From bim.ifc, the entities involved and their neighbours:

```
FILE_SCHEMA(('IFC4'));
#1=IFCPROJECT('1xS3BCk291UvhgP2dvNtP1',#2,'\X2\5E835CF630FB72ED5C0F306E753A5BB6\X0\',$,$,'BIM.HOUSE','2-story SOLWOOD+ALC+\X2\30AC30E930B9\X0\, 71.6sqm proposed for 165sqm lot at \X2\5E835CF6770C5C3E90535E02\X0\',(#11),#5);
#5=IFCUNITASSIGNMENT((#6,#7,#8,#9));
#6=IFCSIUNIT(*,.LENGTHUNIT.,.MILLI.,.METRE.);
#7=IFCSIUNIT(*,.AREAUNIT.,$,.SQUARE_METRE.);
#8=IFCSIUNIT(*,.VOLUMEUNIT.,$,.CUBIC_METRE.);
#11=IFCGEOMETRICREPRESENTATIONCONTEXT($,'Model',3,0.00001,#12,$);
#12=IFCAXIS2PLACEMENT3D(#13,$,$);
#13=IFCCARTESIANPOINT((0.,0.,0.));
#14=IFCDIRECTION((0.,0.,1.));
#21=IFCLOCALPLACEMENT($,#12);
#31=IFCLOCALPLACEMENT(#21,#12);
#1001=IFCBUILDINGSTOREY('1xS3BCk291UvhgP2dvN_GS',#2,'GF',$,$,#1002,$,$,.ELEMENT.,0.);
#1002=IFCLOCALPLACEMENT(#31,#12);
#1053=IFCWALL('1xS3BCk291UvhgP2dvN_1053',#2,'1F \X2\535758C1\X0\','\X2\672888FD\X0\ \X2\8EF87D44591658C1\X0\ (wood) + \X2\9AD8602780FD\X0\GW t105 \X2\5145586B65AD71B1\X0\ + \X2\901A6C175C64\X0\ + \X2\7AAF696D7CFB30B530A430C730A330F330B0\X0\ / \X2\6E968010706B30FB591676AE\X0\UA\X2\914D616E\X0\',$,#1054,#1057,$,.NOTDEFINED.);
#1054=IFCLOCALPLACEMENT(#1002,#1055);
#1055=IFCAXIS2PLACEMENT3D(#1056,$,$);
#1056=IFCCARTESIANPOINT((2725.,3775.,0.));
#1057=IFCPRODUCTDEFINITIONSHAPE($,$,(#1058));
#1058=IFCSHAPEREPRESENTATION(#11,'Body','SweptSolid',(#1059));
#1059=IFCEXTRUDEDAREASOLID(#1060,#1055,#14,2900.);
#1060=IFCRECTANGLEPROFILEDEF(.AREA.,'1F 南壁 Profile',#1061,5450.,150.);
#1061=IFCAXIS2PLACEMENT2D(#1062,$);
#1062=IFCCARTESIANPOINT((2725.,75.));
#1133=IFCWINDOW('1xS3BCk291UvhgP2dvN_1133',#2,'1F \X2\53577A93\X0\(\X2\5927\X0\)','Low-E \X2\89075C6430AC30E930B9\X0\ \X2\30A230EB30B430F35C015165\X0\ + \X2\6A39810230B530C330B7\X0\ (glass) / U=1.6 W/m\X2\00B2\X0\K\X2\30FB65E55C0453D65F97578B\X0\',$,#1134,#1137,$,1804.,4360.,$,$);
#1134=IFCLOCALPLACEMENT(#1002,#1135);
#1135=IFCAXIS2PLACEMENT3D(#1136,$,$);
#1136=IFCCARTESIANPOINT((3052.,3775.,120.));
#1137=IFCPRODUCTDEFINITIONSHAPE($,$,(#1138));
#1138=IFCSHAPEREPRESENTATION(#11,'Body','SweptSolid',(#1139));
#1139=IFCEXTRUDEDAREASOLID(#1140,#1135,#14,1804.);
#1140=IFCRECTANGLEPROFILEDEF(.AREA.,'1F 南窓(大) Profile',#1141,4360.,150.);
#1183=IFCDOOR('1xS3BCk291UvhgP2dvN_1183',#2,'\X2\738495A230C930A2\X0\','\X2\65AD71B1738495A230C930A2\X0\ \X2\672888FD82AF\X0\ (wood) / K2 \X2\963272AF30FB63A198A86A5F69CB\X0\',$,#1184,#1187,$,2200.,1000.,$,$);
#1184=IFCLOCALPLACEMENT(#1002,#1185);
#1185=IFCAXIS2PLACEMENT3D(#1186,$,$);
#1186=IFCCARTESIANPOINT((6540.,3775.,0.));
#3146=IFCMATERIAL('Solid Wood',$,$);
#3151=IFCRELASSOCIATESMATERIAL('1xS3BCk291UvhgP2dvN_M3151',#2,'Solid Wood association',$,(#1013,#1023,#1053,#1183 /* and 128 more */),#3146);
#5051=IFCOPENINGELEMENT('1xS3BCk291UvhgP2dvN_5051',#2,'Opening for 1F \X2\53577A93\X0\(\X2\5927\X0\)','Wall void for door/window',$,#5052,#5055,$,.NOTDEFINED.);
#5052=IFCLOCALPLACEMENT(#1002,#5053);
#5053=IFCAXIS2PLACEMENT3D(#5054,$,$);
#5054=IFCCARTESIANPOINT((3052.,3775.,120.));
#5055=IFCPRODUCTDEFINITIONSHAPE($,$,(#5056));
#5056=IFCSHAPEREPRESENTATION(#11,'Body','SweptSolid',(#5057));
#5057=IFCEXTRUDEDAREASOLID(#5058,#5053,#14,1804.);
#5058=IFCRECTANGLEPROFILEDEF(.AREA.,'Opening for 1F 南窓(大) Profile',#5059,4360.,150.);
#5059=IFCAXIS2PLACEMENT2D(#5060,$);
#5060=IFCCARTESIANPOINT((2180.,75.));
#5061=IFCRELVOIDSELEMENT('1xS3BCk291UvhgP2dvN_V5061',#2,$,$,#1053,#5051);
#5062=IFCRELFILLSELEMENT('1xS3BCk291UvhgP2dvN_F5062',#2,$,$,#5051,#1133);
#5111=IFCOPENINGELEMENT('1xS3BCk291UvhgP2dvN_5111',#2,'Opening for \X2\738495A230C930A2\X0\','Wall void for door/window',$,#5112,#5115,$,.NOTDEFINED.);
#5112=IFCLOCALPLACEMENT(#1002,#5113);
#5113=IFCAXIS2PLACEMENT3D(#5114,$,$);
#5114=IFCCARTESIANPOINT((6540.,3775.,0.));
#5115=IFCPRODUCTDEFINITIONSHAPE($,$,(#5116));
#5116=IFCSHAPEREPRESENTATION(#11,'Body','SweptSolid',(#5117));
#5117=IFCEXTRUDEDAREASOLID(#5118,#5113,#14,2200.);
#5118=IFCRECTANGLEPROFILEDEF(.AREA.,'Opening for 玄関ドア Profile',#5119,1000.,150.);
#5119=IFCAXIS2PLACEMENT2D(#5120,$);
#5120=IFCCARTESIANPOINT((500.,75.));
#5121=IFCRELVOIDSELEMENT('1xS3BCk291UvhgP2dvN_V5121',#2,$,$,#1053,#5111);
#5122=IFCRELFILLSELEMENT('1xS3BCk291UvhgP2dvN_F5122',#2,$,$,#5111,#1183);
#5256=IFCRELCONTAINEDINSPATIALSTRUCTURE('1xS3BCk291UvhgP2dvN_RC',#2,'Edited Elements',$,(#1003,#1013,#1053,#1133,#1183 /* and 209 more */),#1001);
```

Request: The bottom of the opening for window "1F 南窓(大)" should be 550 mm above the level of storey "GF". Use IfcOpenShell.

```python
import numpy as np
import ifcopenshell
import ifcopenshell.api.geometry
import ifcopenshell.geom
import ifcopenshell.util.element
import ifcopenshell.util.placement
import ifcopenshell.util.shape
import ifcopenshell.util.unit

model = ifcopenshell.open("bim.ifc")
unit_scale = ifcopenshell.util.unit.calculate_unit_scale(model)

window = model.by_guid("1xS3BCk291UvhgP2dvN_1133")
opening = window.FillsVoids[0].RelatingOpeningElement
storey = ifcopenshell.util.element.get_container(window, ifc_class="IfcBuildingStorey")
level = ifcopenshell.util.placement.get_local_placement(storey.ObjectPlacement)[2, 3]

# The opening's origin need not be at the sill, so measure its lowest point.
shape = ifcopenshell.geom.create_shape(ifcopenshell.geom.settings(), opening)
bottom = ifcopenshell.util.shape.get_shape_bottom_elevation(shape, shape.geometry) / unit_scale
dz = level + 0.55 / unit_scale - bottom

shift = np.array([0.0, 0.0, dz])
# The window is not placed relative to its opening, so move both.
for product in (opening, window):
    matrix = ifcopenshell.util.placement.get_local_placement(product.ObjectPlacement)
    matrix[:3, 3] += shift
    ifcopenshell.api.geometry.edit_object_placement(model, product=product, matrix=matrix, is_si=False)

print(f"moved by {dz * unit_scale:+.3f} m")

model.write("bim_updated.ifc")
```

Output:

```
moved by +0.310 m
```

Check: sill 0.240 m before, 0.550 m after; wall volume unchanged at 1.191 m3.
